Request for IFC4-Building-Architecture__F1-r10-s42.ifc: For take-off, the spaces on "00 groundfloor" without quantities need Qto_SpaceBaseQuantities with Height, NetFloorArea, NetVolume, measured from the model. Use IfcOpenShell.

First a look at what the model holds.

```python
import ifcopenshell
import ifcopenshell.util.element
import ifcopenshell.util.unit

model = ifcopenshell.open("IFC4-Building-Architecture__F1-r10-s42.ifc")
print(model.schema)
for unit_type in ("LENGTHUNIT", "AREAUNIT", "VOLUMEUNIT"):
    print(unit_type, ifcopenshell.util.unit.calculate_unit_scale(model, unit_type))
storey = next(s for s in model.by_type("IfcBuildingStorey") if s.Name == "00 groundfloor")
spaces = [e for e in ifcopenshell.util.element.get_decomposition(storey) if e.is_a("IfcSpace")]
for e in sorted(spaces, key=lambda e: e.id()):
    print(e.id(), e.is_a(), e.Name, list(ifcopenshell.util.element.get_psets(e, qtos_only=True)), sep=" | ")
```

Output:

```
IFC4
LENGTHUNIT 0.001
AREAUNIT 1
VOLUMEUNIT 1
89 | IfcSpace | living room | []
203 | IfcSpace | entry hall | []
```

```python
import ifcopenshell
import ifcopenshell.api.pset
import ifcopenshell.geom
import ifcopenshell.util.element
import ifcopenshell.util.shape
import ifcopenshell.util.unit

model = ifcopenshell.open("IFC4-Building-Architecture__F1-r10-s42.ifc")
unit_scale = ifcopenshell.util.unit.calculate_unit_scale(model)
area_scale = ifcopenshell.util.unit.calculate_unit_scale(model, "AREAUNIT")
volume_scale = ifcopenshell.util.unit.calculate_unit_scale(model, "VOLUMEUNIT")
settings = ifcopenshell.geom.settings()

storey = next(s for s in model.by_type("IfcBuildingStorey") if s.Name == "00 groundfloor")
spaces = [e for e in ifcopenshell.util.element.get_decomposition(storey) if e.is_a("IfcSpace")]

for e in sorted(spaces, key=lambda e: e.id()):
    if ifcopenshell.util.element.get_psets(e, qtos_only=True, should_inherit=False):
        continue
    # Geometry comes back in metres, in the element's own axes.
    shape = ifcopenshell.geom.create_shape(settings, e)
    values = {
        "Height": ifcopenshell.util.shape.get_z(shape.geometry) / unit_scale,
        "NetFloorArea": ifcopenshell.util.shape.get_footprint_area(shape.geometry) / area_scale,
        "NetVolume": ifcopenshell.util.shape.get_volume(shape.geometry) / volume_scale,
    }
    qto = ifcopenshell.api.pset.add_qto(model, product=e, name="Qto_SpaceBaseQuantities")
    ifcopenshell.api.pset.edit_qto(model, qto=qto, properties=values)
    print(e.id(), {k: round(v, 3) for k, v in values.items()})

model.write("IFC4-Building-Architecture__F1-r10-s42-out.ifc")
```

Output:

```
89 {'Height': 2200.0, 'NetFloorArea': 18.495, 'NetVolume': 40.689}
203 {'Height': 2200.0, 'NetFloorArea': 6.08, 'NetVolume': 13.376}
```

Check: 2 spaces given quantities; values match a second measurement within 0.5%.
